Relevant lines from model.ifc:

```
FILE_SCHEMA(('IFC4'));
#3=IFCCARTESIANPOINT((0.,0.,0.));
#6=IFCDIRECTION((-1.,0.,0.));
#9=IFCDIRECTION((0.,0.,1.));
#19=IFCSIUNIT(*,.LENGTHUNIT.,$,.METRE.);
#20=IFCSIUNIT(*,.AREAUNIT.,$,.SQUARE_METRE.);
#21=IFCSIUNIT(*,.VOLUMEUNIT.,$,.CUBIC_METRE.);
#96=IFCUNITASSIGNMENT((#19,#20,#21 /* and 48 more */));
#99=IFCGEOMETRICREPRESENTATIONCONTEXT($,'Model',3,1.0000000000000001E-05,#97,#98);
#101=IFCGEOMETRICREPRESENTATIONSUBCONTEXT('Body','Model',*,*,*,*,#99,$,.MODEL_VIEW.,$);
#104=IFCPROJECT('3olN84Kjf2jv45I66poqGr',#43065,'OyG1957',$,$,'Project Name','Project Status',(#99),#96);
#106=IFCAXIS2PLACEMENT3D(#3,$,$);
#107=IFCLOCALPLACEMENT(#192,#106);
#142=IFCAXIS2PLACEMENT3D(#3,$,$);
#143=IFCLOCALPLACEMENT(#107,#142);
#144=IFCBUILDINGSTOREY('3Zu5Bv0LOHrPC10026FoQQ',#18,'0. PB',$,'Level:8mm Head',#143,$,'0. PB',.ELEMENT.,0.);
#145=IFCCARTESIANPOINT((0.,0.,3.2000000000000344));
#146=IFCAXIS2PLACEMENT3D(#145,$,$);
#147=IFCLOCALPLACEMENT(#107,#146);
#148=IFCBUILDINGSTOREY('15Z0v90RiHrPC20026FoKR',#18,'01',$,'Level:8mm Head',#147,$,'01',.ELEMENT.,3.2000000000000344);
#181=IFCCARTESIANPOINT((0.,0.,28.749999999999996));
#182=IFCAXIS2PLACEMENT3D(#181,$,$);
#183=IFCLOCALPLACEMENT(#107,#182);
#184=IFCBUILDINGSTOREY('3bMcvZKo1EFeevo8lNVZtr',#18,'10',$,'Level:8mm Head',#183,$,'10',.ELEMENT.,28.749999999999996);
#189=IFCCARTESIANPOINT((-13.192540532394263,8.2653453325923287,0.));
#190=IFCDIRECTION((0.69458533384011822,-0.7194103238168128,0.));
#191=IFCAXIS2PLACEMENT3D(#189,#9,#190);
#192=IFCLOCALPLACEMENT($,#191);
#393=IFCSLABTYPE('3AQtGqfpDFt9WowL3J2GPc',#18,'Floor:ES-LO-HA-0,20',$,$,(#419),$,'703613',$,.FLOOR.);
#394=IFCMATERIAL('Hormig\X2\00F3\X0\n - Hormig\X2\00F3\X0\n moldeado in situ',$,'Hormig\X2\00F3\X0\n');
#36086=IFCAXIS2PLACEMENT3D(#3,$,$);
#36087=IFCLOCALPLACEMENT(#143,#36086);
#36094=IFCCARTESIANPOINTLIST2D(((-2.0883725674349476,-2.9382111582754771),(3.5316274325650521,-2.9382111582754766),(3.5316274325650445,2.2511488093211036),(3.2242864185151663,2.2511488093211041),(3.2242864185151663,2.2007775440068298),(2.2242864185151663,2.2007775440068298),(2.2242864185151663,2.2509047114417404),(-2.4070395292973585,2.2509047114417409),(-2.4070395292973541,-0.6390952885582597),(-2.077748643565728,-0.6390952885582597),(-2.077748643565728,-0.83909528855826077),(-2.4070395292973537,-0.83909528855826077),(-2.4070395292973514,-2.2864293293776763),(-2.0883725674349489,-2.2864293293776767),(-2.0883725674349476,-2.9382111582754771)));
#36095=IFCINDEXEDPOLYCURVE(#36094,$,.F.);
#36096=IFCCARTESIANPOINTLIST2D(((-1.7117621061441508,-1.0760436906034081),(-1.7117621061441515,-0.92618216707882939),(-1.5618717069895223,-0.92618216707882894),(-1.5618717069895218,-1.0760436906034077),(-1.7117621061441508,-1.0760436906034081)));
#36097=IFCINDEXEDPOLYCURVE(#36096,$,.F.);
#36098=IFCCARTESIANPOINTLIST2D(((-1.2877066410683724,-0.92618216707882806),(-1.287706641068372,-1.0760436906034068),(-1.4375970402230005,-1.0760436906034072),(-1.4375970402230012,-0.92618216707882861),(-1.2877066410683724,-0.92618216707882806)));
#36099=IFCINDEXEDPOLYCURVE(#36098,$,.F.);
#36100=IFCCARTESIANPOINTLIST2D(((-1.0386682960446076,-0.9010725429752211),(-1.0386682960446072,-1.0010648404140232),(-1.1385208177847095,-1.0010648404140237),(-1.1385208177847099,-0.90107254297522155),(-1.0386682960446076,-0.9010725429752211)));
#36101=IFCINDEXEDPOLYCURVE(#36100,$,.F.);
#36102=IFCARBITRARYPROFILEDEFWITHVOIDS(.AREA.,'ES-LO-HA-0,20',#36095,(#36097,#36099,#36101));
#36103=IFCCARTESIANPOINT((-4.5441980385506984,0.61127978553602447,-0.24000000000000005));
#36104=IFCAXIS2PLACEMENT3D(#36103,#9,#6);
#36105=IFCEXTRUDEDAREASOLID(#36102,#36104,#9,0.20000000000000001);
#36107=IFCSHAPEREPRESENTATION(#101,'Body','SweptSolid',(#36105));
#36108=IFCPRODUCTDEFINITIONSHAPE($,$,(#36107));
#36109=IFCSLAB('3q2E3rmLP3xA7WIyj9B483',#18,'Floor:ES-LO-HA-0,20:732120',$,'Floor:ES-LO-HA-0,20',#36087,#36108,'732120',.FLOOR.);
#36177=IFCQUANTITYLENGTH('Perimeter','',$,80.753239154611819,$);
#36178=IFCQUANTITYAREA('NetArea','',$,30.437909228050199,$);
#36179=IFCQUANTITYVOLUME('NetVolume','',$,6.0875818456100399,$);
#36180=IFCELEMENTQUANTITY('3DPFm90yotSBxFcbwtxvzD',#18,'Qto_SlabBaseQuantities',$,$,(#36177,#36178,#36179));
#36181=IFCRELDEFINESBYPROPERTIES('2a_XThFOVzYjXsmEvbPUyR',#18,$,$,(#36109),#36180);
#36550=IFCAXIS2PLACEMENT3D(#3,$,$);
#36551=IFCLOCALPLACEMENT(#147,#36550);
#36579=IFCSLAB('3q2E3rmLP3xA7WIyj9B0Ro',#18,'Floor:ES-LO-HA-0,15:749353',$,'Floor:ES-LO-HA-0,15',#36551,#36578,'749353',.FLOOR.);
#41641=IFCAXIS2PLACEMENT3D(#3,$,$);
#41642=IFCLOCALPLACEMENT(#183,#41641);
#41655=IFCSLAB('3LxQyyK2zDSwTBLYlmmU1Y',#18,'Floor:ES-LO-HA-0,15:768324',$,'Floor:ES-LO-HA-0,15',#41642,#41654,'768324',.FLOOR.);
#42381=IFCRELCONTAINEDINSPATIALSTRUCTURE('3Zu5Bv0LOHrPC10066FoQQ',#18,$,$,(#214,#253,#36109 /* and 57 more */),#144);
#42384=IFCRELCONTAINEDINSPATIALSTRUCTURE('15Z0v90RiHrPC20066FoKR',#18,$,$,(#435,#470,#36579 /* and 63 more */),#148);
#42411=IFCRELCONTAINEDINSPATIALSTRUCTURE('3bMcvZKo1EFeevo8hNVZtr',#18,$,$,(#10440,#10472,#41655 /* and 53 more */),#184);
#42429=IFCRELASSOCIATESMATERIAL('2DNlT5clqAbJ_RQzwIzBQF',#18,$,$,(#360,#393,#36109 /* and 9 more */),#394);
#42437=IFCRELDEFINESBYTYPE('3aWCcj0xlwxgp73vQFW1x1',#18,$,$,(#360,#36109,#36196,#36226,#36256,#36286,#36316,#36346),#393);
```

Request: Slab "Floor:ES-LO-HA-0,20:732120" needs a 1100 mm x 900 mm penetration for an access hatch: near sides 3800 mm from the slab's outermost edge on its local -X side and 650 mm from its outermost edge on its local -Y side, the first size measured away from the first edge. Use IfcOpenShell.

```python
import numpy as np
import ifcopenshell
import ifcopenshell.api.feature
import ifcopenshell.api.geometry
import ifcopenshell.api.pset
import ifcopenshell.api.root
import ifcopenshell.geom
import ifcopenshell.util.element
import ifcopenshell.util.placement
import ifcopenshell.util.representation
import ifcopenshell.util.shape
import ifcopenshell.util.unit

model = ifcopenshell.open("model.ifc")
unit_scale = ifcopenshell.util.unit.calculate_unit_scale(model)
area_scale = ifcopenshell.util.unit.calculate_unit_scale(model, "AREAUNIT")
volume_scale = ifcopenshell.util.unit.calculate_unit_scale(model, "VOLUMEUNIT")
settings = ifcopenshell.geom.settings()


def volume(element):
    """Net volume in cubic metres, openings subtracted."""
    shape = ifcopenshell.geom.create_shape(settings, element)
    return ifcopenshell.util.shape.get_volume(shape.geometry)


slab = model.by_guid("3q2E3rmLP3xA7WIyj9B483")
before = volume(slab)

# Extent in the slab's own axes, in metres. The edges named are its -X and -Y sides.
slab_shape = ifcopenshell.geom.create_shape(settings, slab)
vertices = ifcopenshell.util.shape.get_vertices(slab_shape.geometry)
x_min, y_min, bottom = vertices.min(axis=0)
top = vertices[:, 2].max()

opening = ifcopenshell.api.root.create_entity(model, ifc_class="IfcOpeningElement", name="Access hatch opening", predefined_type="OPENING")
context = ifcopenshell.util.representation.get_context(model, "Model", "Body", "MODEL_VIEW")
width, depth = 1.1, 0.9
outline = [(0.0, 0.0), (width, 0.0), (width, depth), (0.0, depth), (0.0, 0.0)]
# Overshoot both faces by 50 mm so the cut is clean.
shape = ifcopenshell.api.geometry.add_slab_representation(
    model, context=context, depth=top - bottom + 0.1, polyline=outline
)
ifcopenshell.api.geometry.assign_representation(model, product=opening, representation=shape)

matrix = ifcopenshell.util.placement.get_local_placement(slab.ObjectPlacement)
matrix[:, 3] = matrix @ np.append(np.array([x_min + 3.8, y_min + 0.65, bottom - 0.05]) / unit_scale, 1.0)
ifcopenshell.api.geometry.edit_object_placement(model, product=opening, matrix=matrix, is_si=False)
ifcopenshell.api.feature.add_feature(model, feature=opening, element=slab)

after = volume(slab)

# Update the slab's stored quantities.
qto = model.by_id(ifcopenshell.util.element.get_pset(slab, "Qto_SlabBaseQuantities", should_inherit=False)["id"])
ifcopenshell.api.pset.edit_qto(model, qto=qto, properties={
    "NetArea": after / (top - bottom) / area_scale,
    "NetVolume": after / volume_scale,
})

print(f"slab volume {before:.3f} -> {after:.3f} m3")

model.write("model-out.ifc")
```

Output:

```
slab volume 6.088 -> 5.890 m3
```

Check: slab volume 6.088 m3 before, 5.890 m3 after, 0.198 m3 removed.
